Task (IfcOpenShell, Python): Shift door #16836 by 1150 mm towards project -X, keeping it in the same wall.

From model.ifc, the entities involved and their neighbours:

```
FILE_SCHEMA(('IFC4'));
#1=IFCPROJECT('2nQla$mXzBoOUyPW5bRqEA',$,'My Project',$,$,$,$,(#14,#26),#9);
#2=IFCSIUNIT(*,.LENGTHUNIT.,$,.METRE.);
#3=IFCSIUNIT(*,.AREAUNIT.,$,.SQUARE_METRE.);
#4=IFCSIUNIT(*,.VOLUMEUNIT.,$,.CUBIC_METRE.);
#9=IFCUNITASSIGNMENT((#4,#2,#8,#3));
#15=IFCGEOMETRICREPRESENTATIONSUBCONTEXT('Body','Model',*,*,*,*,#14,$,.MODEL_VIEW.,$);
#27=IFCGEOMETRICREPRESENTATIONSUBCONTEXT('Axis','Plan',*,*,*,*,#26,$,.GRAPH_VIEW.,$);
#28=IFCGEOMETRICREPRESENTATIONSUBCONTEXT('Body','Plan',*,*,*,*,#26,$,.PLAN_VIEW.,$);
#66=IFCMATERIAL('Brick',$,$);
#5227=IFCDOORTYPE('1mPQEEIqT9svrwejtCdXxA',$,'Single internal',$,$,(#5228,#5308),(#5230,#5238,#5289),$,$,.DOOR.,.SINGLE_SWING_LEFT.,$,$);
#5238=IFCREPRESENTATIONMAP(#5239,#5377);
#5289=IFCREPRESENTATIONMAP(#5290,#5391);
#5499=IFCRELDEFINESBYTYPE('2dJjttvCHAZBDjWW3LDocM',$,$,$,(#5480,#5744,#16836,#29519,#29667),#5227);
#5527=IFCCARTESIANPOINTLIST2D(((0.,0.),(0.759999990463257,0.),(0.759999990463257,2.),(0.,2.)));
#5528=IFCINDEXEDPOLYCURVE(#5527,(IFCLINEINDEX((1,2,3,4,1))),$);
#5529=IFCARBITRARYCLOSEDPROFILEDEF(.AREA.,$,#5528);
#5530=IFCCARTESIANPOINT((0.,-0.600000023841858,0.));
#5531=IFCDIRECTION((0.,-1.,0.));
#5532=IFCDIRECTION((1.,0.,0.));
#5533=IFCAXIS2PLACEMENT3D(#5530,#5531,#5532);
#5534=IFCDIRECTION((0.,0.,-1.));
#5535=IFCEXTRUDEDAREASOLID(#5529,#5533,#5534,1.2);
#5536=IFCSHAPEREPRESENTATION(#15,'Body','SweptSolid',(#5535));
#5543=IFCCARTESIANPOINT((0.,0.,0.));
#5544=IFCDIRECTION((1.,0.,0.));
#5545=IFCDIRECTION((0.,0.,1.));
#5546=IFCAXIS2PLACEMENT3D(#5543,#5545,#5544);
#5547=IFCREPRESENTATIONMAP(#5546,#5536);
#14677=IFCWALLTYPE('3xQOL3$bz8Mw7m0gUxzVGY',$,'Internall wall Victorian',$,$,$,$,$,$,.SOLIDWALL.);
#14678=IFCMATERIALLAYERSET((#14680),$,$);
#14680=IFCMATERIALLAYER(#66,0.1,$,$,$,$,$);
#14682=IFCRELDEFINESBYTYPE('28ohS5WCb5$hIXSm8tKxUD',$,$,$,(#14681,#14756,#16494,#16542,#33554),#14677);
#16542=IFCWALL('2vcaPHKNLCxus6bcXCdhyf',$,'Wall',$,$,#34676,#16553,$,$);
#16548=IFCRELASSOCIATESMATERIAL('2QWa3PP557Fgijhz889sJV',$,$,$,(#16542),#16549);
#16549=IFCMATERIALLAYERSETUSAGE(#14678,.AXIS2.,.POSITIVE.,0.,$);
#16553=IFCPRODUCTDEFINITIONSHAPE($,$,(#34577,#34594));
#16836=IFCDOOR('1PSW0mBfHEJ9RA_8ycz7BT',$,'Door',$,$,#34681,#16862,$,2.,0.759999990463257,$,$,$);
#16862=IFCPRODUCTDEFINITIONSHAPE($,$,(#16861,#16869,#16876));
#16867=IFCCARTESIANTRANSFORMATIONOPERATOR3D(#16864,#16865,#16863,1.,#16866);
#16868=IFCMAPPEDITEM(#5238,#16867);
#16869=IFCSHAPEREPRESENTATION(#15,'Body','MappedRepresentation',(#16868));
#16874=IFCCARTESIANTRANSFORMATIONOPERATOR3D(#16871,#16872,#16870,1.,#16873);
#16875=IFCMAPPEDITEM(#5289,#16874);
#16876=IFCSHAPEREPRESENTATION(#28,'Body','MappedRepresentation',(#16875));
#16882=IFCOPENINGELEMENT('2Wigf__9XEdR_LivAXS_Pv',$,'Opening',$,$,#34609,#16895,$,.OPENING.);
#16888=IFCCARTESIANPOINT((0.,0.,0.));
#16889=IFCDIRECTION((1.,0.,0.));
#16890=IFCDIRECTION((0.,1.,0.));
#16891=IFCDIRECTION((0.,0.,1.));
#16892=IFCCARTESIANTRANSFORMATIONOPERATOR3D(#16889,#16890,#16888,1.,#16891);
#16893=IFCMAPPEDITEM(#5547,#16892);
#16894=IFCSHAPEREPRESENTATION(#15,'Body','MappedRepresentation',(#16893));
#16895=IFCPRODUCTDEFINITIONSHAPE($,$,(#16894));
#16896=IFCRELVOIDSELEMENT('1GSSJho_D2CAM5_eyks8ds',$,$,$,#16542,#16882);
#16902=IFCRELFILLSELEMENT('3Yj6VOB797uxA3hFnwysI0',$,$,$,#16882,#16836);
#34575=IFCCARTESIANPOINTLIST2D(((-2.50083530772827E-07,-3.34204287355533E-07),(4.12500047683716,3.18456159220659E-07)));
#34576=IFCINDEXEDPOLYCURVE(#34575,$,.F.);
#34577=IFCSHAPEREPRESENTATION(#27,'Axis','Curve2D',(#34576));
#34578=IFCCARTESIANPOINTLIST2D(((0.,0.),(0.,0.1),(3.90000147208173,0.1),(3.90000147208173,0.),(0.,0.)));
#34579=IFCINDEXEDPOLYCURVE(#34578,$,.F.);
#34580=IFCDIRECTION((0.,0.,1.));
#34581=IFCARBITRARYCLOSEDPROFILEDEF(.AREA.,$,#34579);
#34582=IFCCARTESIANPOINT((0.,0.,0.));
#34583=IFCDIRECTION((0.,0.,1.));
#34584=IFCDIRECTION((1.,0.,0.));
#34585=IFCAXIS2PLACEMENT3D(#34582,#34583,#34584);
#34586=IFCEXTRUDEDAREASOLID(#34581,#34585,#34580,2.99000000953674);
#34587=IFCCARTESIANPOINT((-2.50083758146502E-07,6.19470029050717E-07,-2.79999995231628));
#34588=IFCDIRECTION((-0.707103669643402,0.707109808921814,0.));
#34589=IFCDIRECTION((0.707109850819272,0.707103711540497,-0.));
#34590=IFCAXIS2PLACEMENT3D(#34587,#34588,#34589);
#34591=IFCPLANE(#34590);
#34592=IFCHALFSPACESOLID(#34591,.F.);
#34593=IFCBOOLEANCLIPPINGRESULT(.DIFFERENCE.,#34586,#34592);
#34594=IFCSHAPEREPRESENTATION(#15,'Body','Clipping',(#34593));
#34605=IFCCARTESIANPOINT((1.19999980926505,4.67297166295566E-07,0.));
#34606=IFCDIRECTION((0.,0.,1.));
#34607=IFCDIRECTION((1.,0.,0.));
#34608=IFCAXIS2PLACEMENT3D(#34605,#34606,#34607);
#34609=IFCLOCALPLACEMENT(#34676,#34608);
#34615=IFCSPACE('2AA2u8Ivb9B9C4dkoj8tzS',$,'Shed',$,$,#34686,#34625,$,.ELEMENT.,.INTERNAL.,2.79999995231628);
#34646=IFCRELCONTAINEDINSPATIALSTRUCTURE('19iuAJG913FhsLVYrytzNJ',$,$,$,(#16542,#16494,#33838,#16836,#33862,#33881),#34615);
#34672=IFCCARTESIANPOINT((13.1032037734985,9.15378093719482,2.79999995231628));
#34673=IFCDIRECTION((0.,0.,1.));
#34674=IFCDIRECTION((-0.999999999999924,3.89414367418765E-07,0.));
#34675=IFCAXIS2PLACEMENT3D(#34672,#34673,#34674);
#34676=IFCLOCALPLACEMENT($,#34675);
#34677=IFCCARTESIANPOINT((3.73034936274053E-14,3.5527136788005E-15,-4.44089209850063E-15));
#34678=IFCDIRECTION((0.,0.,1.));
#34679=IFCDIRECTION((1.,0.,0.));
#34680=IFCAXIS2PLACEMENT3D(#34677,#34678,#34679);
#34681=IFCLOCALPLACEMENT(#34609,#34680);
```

```python
import ifcopenshell
import ifcopenshell.api.geometry
import ifcopenshell.util.placement
import ifcopenshell.util.unit

model = ifcopenshell.open("model.ifc")
unit_scale = ifcopenshell.util.unit.calculate_unit_scale(model)

door = model.by_guid("1PSW0mBfHEJ9RA_8ycz7BT")
opening = door.FillsVoids[0].RelatingOpeningElement
wall = opening.VoidsElements[0].RelatingBuildingElement

wall_matrix = ifcopenshell.util.placement.get_local_placement(wall.ObjectPlacement)
shift = wall_matrix[:3, 0] * 1.15 / unit_scale
before = ifcopenshell.util.placement.get_local_placement(door.ObjectPlacement)[:3, 3].copy()

# The door is placed relative to its opening, so it follows when the opening moves.
matrix = ifcopenshell.util.placement.get_local_placement(opening.ObjectPlacement)
matrix[:3, 3] += shift
ifcopenshell.api.geometry.edit_object_placement(
    model, product=opening, matrix=matrix, is_si=False, should_transform_children=True
)

after = ifcopenshell.util.placement.get_local_placement(door.ObjectPlacement)[:3, 3]
print("door moved by", (after - before).round(3) + 0.0)

model.write("model-out.ifc")
```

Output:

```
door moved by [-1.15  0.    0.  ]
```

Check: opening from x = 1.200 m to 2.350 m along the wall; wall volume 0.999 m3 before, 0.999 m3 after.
